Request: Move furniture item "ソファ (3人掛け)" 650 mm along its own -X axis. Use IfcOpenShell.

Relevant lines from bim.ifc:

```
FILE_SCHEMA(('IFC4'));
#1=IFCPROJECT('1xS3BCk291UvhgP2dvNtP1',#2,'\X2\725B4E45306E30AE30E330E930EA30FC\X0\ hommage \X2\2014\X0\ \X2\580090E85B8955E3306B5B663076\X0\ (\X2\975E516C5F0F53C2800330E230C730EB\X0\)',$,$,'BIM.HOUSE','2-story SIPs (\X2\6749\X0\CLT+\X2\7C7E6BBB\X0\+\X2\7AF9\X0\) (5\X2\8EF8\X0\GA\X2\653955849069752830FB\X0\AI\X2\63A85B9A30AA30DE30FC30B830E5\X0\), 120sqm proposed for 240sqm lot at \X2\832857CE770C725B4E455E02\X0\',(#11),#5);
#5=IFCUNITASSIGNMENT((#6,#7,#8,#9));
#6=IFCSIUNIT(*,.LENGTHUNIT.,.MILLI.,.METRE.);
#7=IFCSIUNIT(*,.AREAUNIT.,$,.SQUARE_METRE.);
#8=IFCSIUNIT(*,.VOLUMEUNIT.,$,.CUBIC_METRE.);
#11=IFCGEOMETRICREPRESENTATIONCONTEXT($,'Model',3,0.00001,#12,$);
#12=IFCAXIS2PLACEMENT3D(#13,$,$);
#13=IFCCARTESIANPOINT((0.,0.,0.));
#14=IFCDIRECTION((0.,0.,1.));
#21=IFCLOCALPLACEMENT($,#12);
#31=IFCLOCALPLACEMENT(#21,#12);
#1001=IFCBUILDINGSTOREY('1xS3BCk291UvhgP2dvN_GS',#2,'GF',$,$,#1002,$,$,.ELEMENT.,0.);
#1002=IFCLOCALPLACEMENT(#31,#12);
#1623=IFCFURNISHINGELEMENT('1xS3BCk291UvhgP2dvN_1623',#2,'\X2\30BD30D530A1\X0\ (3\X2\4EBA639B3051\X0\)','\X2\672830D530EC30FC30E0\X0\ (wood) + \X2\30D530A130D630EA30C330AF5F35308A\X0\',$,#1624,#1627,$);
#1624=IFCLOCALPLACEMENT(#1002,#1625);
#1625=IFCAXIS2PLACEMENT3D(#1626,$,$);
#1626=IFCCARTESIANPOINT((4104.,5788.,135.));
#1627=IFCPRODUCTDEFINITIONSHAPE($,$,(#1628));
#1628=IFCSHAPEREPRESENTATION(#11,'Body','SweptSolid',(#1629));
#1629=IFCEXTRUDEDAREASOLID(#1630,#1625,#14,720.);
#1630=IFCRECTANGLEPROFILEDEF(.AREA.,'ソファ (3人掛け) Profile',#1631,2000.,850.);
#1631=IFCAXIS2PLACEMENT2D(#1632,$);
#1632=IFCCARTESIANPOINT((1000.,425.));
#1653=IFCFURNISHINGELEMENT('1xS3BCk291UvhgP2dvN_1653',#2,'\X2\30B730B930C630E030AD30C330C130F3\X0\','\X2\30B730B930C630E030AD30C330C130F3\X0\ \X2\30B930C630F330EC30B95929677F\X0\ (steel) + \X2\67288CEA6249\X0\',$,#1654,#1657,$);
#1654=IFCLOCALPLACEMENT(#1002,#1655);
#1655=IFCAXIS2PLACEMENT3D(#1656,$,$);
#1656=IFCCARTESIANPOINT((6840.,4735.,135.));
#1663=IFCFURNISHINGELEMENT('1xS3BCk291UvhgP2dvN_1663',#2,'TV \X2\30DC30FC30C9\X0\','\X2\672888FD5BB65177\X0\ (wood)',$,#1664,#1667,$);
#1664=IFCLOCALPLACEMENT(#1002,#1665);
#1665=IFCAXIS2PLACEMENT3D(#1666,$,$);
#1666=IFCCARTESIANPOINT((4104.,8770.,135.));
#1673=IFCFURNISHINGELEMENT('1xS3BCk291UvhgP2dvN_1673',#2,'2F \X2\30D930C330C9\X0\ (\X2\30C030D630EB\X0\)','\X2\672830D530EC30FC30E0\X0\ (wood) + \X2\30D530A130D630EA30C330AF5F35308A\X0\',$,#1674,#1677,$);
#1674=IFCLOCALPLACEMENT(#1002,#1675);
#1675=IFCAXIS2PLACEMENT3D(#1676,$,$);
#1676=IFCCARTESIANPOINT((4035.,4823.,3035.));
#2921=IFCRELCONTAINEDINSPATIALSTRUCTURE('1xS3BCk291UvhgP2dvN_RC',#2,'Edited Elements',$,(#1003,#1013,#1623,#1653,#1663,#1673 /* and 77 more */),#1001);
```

```python
import ifcopenshell
import ifcopenshell.api.geometry
import ifcopenshell.util.placement

model = ifcopenshell.open("bim.ifc")

item = model.by_guid("1xS3BCk291UvhgP2dvN_1623")
matrix = ifcopenshell.util.placement.get_local_placement(item.ObjectPlacement)
matrix[:3, 3] -= matrix[:3, 0] * 650.0
ifcopenshell.api.geometry.edit_object_placement(model, product=item, matrix=matrix, is_si=False)

print(ifcopenshell.util.placement.get_local_placement(item.ObjectPlacement).round(3) + 0.0)

model.write("bim_v2.ifc")
```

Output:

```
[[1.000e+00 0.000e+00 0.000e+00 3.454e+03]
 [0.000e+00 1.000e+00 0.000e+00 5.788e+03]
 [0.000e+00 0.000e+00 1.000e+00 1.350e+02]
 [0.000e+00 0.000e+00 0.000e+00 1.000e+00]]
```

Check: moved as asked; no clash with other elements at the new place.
